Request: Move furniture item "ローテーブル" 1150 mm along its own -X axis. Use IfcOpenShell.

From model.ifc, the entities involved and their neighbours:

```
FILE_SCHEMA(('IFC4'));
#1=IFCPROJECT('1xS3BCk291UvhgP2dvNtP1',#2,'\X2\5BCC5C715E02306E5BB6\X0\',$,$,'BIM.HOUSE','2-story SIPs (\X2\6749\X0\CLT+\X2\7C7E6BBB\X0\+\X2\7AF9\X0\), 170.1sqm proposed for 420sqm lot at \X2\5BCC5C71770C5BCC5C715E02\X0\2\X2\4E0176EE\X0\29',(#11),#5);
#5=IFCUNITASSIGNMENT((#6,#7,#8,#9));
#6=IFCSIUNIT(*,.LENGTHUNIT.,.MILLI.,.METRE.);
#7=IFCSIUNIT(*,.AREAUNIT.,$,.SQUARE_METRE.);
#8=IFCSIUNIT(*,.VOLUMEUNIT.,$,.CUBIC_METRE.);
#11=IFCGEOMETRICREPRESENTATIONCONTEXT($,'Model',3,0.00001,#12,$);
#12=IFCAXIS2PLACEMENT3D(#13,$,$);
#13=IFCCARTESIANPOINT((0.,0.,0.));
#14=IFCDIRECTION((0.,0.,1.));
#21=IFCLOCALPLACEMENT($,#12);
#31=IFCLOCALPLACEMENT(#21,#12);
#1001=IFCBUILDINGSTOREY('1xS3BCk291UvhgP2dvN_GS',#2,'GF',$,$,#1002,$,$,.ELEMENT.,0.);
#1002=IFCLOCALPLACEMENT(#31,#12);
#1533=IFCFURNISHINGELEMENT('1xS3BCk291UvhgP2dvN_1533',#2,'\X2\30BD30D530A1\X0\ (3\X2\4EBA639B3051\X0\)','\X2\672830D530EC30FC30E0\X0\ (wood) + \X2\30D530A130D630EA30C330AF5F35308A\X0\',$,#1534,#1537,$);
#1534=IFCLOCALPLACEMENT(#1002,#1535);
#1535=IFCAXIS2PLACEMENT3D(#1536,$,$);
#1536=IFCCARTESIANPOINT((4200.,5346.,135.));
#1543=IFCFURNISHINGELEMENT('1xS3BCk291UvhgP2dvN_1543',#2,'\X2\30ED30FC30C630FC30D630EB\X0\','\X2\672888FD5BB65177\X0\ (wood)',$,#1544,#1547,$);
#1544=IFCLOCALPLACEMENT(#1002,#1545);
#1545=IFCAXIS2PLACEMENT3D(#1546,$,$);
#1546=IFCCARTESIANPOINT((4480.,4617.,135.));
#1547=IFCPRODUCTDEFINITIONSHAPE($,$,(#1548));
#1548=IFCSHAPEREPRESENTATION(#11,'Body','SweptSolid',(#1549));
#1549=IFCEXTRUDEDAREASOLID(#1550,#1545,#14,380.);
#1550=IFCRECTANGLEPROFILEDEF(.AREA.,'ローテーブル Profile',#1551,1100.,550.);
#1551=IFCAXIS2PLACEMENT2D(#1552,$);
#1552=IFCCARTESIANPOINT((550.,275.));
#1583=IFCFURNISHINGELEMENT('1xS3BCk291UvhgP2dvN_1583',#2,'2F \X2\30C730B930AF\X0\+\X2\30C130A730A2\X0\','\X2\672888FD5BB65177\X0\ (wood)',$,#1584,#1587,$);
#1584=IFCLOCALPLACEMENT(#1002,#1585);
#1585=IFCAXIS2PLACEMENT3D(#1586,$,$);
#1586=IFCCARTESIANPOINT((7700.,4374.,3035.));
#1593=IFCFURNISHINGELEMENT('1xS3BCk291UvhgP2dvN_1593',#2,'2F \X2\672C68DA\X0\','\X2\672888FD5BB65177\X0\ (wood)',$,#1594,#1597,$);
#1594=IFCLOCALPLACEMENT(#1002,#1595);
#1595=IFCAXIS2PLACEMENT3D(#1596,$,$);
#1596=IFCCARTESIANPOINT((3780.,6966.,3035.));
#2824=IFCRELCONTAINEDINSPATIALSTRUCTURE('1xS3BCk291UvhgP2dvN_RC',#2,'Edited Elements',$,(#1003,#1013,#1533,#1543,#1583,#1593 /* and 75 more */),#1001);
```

```python
import ifcopenshell
import ifcopenshell.api.geometry
import ifcopenshell.util.placement
import ifcopenshell.util.unit

model = ifcopenshell.open("model.ifc")
unit_scale = ifcopenshell.util.unit.calculate_unit_scale(model)

item = model.by_guid("1xS3BCk291UvhgP2dvN_1543")
matrix = ifcopenshell.util.placement.get_local_placement(item.ObjectPlacement)
matrix[:3, 3] -= matrix[:3, 0] * 1.15 / unit_scale
ifcopenshell.api.geometry.edit_object_placement(model, product=item, matrix=matrix, is_si=False)

print(ifcopenshell.util.placement.get_local_placement(item.ObjectPlacement).round(3) + 0.0)

model.write("model_rev.ifc")
```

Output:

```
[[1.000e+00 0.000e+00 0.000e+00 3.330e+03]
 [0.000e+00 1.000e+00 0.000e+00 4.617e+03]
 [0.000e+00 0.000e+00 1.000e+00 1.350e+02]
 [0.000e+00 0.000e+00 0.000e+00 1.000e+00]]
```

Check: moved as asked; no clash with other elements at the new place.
